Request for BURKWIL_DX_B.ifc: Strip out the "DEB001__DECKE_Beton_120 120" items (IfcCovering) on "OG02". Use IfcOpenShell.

First a look at what the model holds.

```python
import ifcopenshell
import ifcopenshell.util.element

model = ifcopenshell.open("BURKWIL_DX_B.ifc")
print(model.schema)
storey = next(s for s in model.by_type("IfcBuildingStorey") if s.Name == "OG02")
coverings = [e for e in ifcopenshell.util.element.get_decomposition(storey) if e.is_a("IfcCovering")]
seen = {}
for e in coverings:
    element_type = ifcopenshell.util.element.get_type(e)
    name = element_type.Name if element_type not in (None, e) else None
    seen[name] = seen.get(name, 0) + 1
for name, count in sorted(seen.items(), key=str):
    print(count, "x", name)
```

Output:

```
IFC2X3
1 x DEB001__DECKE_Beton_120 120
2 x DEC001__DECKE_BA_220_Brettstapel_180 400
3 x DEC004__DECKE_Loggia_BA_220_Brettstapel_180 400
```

```python
import ifcopenshell
import ifcopenshell.api.root
import ifcopenshell.util.element

model = ifcopenshell.open("BURKWIL_DX_B.ifc")

storey = next(s for s in model.by_type("IfcBuildingStorey") if s.Name == "OG02")
coverings = [e for e in ifcopenshell.util.element.get_decomposition(storey) if e.is_a("IfcCovering")]
targets = [e for e in coverings if (t := ifcopenshell.util.element.get_type(e)) not in (None, e) and t.Name == "DEB001__DECKE_Beton_120 120"]

for e in targets:
    ifcopenshell.api.root.remove_product(model, product=e)
print(len(targets), "removed")

model.write("BURKWIL_DX_B_v2.ifc")
```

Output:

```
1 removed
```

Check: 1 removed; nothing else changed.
